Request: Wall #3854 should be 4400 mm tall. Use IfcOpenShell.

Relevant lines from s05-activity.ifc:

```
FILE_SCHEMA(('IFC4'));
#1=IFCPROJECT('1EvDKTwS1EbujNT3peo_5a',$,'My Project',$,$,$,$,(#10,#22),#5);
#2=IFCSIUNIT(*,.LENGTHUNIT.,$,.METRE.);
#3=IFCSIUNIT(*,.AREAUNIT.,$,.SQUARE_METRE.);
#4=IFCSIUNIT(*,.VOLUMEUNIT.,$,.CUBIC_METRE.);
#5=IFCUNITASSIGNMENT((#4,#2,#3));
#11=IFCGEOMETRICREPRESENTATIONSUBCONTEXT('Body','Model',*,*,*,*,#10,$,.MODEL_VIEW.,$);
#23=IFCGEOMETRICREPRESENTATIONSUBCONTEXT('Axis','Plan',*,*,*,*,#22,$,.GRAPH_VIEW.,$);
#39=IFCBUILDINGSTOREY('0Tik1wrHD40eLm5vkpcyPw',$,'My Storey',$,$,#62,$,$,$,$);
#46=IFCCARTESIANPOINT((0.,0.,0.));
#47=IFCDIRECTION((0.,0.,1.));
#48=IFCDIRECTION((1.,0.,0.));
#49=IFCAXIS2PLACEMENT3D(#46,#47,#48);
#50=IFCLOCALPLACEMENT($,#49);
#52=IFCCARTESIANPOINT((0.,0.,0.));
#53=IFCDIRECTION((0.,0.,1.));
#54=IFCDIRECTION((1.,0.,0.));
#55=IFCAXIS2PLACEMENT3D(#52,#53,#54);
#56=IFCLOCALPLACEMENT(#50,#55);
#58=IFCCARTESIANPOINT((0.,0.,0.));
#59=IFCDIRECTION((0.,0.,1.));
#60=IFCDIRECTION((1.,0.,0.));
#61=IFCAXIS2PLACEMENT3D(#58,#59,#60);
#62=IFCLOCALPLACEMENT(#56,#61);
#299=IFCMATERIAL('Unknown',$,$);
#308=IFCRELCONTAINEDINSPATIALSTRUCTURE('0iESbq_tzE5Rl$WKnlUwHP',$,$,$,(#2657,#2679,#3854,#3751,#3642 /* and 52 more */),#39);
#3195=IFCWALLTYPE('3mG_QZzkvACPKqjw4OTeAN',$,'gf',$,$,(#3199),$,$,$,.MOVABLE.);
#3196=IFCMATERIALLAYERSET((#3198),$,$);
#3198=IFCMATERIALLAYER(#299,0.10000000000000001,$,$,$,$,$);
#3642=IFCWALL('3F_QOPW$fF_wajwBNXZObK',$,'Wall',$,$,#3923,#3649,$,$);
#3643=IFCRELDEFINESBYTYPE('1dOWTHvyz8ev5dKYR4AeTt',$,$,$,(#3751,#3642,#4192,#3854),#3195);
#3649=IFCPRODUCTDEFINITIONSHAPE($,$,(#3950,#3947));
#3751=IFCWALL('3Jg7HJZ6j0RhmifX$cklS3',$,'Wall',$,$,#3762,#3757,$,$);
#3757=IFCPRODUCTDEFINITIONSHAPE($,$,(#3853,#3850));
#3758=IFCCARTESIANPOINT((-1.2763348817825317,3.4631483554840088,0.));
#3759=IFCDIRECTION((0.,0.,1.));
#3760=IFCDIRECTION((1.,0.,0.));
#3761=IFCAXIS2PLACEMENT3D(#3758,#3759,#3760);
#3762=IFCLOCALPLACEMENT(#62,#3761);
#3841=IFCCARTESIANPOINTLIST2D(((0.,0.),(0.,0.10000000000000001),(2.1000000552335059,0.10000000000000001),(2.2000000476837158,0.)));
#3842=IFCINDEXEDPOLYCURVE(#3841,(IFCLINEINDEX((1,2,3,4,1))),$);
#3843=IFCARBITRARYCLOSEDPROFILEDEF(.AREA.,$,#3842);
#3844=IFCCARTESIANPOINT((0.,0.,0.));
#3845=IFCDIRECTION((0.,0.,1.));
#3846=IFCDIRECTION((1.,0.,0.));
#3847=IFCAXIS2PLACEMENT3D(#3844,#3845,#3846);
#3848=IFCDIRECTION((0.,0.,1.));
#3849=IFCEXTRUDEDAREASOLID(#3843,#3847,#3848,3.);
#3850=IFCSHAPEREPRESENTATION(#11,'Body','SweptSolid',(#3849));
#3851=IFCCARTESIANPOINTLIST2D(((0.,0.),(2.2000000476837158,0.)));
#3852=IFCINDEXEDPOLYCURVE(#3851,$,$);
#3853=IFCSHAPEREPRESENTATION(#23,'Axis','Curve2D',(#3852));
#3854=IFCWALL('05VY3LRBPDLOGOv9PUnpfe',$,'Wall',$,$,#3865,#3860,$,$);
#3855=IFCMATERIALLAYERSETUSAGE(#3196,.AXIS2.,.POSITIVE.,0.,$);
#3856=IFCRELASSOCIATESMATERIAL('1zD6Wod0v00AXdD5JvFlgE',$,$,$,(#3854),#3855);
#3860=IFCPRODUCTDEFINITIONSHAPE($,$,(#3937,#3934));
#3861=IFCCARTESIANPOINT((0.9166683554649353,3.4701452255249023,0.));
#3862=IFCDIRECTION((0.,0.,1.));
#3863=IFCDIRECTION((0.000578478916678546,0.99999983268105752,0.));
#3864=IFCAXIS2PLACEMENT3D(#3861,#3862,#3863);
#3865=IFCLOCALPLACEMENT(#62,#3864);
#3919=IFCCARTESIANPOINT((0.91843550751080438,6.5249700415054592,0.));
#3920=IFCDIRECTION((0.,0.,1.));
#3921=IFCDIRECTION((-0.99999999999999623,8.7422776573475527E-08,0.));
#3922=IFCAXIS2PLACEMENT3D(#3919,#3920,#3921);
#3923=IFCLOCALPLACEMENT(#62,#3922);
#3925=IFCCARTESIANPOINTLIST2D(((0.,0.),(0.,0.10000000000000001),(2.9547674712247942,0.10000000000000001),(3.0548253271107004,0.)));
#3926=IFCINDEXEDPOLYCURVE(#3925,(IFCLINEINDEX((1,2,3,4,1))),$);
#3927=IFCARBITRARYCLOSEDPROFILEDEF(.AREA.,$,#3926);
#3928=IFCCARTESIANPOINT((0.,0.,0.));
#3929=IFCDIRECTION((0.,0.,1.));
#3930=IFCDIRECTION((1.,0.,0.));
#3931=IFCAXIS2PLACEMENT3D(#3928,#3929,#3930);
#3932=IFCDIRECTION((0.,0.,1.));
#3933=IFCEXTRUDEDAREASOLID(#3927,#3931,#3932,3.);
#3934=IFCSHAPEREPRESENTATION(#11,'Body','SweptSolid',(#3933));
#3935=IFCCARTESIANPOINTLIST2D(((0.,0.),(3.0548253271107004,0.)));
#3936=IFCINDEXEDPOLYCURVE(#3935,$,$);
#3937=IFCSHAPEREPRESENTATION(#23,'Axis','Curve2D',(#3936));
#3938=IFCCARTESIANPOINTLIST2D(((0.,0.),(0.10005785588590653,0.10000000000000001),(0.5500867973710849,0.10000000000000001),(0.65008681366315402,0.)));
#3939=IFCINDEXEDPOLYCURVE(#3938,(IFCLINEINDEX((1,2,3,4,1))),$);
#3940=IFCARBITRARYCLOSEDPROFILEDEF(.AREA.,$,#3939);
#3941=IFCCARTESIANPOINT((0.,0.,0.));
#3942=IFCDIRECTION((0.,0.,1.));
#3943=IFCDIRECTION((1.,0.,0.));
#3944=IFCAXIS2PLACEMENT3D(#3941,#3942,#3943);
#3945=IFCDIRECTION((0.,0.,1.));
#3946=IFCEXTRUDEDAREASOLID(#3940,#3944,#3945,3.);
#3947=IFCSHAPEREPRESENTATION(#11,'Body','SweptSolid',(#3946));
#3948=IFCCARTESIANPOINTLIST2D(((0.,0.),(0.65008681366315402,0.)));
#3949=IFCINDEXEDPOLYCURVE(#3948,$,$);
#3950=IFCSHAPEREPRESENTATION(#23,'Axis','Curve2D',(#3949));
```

```python
import ifcopenshell
import ifcopenshell.geom
import ifcopenshell.util.representation
import ifcopenshell.util.shape

model = ifcopenshell.open("s05-activity.ifc")
settings = ifcopenshell.geom.settings()


def volume(element):
    """Net volume in cubic metres, openings subtracted."""
    shape = ifcopenshell.geom.create_shape(settings, element)
    return ifcopenshell.util.shape.get_volume(shape.geometry)


wall = model.by_id(3854)
before = volume(wall)

body = ifcopenshell.util.representation.get_representation(wall, "Model", "Body")
solid = body.Items[0]
old_height = solid.Depth
solid.Depth = 4.4
after = volume(wall)

print(f"height {old_height:g} -> {solid.Depth:g}, volume {before:.3f} -> {after:.3f} m3")

model.write("s05-activity_edited.ifc")
```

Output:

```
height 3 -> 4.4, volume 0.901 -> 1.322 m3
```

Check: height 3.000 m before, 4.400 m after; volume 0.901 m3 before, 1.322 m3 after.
